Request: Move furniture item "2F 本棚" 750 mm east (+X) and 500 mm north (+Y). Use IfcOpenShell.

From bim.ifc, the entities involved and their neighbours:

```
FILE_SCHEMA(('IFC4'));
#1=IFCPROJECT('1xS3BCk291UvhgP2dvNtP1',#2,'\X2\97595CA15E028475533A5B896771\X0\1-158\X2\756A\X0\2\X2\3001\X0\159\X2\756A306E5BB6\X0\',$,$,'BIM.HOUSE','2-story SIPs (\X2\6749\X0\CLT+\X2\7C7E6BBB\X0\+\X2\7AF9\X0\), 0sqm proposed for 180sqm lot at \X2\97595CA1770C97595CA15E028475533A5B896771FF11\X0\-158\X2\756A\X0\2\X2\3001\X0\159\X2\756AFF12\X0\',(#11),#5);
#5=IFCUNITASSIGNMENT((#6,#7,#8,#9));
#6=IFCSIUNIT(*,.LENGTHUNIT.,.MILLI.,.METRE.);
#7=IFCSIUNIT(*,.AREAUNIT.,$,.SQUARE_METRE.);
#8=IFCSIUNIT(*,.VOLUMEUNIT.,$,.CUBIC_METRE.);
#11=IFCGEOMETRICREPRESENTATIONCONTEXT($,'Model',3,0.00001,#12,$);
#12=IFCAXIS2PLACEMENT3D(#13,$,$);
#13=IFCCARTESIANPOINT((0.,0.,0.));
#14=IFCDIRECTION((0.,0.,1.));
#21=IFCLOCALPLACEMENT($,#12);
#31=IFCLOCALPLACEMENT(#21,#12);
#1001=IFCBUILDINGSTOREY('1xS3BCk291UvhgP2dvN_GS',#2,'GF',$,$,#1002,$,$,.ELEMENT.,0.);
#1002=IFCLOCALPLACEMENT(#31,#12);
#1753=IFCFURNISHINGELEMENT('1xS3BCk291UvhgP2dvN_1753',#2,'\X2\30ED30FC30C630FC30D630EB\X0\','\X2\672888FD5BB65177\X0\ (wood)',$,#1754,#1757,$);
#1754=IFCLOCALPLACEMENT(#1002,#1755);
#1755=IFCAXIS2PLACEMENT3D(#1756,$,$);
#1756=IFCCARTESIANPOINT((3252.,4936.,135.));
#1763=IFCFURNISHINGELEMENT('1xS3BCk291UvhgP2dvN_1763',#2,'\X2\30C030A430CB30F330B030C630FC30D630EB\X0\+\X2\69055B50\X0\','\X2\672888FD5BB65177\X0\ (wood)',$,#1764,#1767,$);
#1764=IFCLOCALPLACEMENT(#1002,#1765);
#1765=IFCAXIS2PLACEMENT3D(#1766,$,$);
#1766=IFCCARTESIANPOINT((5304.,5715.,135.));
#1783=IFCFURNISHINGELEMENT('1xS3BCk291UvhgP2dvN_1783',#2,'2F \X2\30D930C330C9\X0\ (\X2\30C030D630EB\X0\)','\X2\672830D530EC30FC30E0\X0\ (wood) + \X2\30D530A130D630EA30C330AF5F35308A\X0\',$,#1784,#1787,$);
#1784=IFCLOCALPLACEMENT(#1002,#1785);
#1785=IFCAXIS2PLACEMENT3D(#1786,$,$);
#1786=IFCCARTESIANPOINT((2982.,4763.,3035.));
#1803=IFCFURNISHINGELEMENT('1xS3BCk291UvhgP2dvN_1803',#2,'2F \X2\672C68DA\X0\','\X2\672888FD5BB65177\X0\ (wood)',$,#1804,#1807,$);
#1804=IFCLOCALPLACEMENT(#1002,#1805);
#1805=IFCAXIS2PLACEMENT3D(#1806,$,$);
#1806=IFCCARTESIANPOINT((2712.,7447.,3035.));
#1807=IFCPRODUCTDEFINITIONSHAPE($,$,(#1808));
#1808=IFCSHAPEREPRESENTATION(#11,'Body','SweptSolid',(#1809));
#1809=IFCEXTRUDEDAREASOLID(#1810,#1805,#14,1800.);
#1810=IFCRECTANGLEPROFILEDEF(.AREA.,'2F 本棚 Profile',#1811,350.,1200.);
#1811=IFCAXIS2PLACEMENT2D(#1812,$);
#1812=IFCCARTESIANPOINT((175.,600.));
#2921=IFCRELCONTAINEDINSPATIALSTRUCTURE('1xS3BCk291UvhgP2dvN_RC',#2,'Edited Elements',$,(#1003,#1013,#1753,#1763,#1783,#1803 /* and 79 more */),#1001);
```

```python
import ifcopenshell
import ifcopenshell.api.geometry
import ifcopenshell.util.placement

model = ifcopenshell.open("bim.ifc")

item = model.by_guid("1xS3BCk291UvhgP2dvN_1803")
matrix = ifcopenshell.util.placement.get_local_placement(item.ObjectPlacement)
matrix[0, 3] += 750.0
matrix[1, 3] += 500.0
ifcopenshell.api.geometry.edit_object_placement(model, product=item, matrix=matrix, is_si=False)

print(ifcopenshell.util.placement.get_local_placement(item.ObjectPlacement).round(3) + 0.0)

model.write("bim_rev.ifc")
```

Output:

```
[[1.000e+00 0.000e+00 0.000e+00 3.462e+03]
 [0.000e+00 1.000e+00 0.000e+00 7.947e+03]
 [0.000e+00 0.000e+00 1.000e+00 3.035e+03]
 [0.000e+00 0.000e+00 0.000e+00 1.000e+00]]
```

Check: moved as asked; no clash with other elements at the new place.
